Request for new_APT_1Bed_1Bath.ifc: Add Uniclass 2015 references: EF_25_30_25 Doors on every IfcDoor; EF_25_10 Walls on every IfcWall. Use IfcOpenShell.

First a look at what the model holds.

```python
import ifcopenshell

model = ifcopenshell.open("new_APT_1Bed_1Bath.ifc")
print(model.schema)
print("classifications:", [c.Name for c in model.by_type("IfcClassification")])
for ifc_class in ("IfcDoor", "IfcRoof", "IfcStair", "IfcWall", "IfcWindow"):
    print(ifc_class, len(model.by_type(ifc_class)))
```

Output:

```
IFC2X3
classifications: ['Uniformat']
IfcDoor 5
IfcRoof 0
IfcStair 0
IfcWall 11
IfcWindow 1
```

```python
import ifcopenshell
import ifcopenshell.api.classification

model = ifcopenshell.open("new_APT_1Bed_1Bath.ifc")

# IFC2X3 requires Source and Edition and has no link from the project to the system.
system = model.create_entity("IfcClassification", Source="NBS", Edition="2015", Name="Uniclass 2015")

codes = {
    "IfcDoor": ("EF_25_30_25", "Doors"),
    "IfcWall": ("EF_25_10", "Walls"),
}
for ifc_class, (code, name) in codes.items():
    products = model.by_type(ifc_class)
    ifcopenshell.api.classification.add_reference(
        model, products=products, classification=system, identification=code, name=name
    )
    print(code, len(products))

model.write("new_APT_1Bed_1Bath_v2.ifc")
```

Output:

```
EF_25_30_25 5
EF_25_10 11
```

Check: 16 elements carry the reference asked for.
